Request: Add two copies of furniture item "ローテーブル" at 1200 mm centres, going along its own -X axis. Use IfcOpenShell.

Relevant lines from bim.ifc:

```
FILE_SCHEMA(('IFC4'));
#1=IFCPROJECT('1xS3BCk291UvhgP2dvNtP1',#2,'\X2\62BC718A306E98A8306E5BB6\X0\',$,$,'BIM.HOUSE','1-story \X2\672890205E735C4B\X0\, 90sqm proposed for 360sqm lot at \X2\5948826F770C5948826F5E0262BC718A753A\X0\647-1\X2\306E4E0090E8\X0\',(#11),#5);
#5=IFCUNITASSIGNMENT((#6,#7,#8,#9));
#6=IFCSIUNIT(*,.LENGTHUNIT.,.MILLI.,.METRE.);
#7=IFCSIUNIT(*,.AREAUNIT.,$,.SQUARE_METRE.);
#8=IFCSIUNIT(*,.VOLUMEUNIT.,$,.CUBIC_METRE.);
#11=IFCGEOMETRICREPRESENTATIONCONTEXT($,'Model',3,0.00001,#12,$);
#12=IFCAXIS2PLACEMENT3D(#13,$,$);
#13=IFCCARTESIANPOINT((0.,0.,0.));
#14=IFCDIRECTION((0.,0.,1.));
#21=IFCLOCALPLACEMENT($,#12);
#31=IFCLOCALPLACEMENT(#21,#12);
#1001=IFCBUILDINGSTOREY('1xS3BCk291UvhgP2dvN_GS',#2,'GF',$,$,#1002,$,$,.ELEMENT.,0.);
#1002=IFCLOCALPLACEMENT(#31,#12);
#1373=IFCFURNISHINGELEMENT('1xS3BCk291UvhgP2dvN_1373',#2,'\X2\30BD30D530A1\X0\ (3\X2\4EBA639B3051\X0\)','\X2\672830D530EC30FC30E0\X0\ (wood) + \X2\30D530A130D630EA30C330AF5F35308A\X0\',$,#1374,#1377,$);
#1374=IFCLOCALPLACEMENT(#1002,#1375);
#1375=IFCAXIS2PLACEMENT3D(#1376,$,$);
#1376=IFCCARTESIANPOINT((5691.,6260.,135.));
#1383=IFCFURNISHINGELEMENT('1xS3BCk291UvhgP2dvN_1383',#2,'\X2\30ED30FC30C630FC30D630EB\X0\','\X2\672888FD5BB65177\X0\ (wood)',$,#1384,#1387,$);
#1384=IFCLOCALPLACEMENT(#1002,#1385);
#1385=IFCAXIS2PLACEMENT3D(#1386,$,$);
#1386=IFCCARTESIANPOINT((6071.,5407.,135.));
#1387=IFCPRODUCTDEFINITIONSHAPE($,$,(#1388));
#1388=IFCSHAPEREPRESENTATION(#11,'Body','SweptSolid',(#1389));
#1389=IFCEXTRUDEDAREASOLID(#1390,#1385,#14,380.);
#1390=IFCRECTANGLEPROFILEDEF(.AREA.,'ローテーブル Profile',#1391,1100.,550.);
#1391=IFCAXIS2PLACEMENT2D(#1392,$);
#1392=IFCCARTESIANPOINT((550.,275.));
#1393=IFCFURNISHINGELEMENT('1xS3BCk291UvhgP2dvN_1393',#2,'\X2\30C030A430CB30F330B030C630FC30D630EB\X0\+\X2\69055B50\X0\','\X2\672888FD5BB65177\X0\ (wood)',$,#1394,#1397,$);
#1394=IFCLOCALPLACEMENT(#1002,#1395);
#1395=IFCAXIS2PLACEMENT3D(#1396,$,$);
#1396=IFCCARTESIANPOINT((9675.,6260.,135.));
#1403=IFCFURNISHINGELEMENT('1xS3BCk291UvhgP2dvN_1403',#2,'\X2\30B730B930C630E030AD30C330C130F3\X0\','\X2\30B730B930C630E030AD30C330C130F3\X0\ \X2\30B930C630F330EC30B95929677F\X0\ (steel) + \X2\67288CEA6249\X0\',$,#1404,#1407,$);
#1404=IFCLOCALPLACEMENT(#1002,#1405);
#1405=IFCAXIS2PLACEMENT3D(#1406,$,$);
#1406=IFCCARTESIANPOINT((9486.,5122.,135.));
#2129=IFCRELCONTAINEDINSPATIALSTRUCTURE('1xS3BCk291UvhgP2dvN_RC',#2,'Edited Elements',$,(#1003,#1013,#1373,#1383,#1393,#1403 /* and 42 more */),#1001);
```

```python
import ifcopenshell
import ifcopenshell.api.geometry
import ifcopenshell.api.root
import ifcopenshell.util.element
import ifcopenshell.util.placement
import ifcopenshell.util.unit

model = ifcopenshell.open("bim.ifc")
unit_scale = ifcopenshell.util.unit.calculate_unit_scale(model)


def reuse_history(source, copy):
    """copy_class also copies each property set's owner history, people and application; keep the originals."""
    for rel in copy.IsDefinedBy:
        if rel.is_a("IfcRelDefinesByProperties") and (history := rel.RelatingPropertyDefinition.OwnerHistory):
            rel.RelatingPropertyDefinition.OwnerHistory = source.OwnerHistory
            ifcopenshell.util.element.remove_deep2(model, history)


source = model.by_id(1383)
base = ifcopenshell.util.placement.get_local_placement(source.ObjectPlacement)
step = -base[:3, 0] * 1.2 / unit_scale

for i in range(1, 3):
    copy = ifcopenshell.api.root.copy_class(model, product=source)
    copy.Representation = ifcopenshell.util.element.copy_deep(
        model, source.Representation, exclude=["IfcGeometricRepresentationContext", "IfcRepresentationMap"]
    )
    reuse_history(source, copy)
    matrix = base.copy()
    matrix[:3, 3] += i * step
    print("added at", matrix[:3, 3].round(3) + 0.0)
    ifcopenshell.api.geometry.edit_object_placement(model, product=copy, matrix=matrix, is_si=False)

model.write("bim_rev.ifc")
```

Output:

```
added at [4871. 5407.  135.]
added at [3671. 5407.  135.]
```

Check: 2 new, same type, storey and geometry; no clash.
